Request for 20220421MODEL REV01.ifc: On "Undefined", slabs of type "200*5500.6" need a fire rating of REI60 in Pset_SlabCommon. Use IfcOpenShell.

First a look at what the model holds.

```python
import ifcopenshell
import ifcopenshell.util.element

model = ifcopenshell.open("20220421MODEL REV01.ifc")
print(model.schema)
storey = next(s for s in model.by_type("IfcBuildingStorey") if s.Name == "Undefined")
slabs = [e for e in ifcopenshell.util.element.get_decomposition(storey) if e.is_a("IfcSlab")]
seen = {}
for e in slabs:
    element_type = ifcopenshell.util.element.get_type(e)
    key = (element_type.Name if element_type != e and element_type else None, ifcopenshell.util.element.get_pset(e, "Pset_SlabCommon", "FireRating"))
    seen[key] = seen.get(key, 0) + 1
for (name, value), count in sorted(seen.items(), key=str):
    print(count, "x", name, "|", value)
```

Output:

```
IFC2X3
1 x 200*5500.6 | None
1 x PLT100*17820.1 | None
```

```python
import ifcopenshell
import ifcopenshell.api.pset
import ifcopenshell.util.element

model = ifcopenshell.open("20220421MODEL REV01.ifc")

storey = next(s for s in model.by_type("IfcBuildingStorey") if s.Name == "Undefined")
slabs = [e for e in ifcopenshell.util.element.get_decomposition(storey) if e.is_a("IfcSlab")]

count = 0
for e in slabs:
    element_type = ifcopenshell.util.element.get_type(e)
    if element_type in (None, e) or element_type.Name != "200*5500.6":
        continue
    # add_pset returns the element's existing set when there is one.
    pset = ifcopenshell.api.pset.add_pset(model, product=e, name="Pset_SlabCommon")
    ifcopenshell.api.pset.edit_pset(model, pset=pset, properties={"FireRating": "REI60"})
    count += 1

print(count, "slabs updated")

model.write("20220421MODEL REV01_v2.ifc")
```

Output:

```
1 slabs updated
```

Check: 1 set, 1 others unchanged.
